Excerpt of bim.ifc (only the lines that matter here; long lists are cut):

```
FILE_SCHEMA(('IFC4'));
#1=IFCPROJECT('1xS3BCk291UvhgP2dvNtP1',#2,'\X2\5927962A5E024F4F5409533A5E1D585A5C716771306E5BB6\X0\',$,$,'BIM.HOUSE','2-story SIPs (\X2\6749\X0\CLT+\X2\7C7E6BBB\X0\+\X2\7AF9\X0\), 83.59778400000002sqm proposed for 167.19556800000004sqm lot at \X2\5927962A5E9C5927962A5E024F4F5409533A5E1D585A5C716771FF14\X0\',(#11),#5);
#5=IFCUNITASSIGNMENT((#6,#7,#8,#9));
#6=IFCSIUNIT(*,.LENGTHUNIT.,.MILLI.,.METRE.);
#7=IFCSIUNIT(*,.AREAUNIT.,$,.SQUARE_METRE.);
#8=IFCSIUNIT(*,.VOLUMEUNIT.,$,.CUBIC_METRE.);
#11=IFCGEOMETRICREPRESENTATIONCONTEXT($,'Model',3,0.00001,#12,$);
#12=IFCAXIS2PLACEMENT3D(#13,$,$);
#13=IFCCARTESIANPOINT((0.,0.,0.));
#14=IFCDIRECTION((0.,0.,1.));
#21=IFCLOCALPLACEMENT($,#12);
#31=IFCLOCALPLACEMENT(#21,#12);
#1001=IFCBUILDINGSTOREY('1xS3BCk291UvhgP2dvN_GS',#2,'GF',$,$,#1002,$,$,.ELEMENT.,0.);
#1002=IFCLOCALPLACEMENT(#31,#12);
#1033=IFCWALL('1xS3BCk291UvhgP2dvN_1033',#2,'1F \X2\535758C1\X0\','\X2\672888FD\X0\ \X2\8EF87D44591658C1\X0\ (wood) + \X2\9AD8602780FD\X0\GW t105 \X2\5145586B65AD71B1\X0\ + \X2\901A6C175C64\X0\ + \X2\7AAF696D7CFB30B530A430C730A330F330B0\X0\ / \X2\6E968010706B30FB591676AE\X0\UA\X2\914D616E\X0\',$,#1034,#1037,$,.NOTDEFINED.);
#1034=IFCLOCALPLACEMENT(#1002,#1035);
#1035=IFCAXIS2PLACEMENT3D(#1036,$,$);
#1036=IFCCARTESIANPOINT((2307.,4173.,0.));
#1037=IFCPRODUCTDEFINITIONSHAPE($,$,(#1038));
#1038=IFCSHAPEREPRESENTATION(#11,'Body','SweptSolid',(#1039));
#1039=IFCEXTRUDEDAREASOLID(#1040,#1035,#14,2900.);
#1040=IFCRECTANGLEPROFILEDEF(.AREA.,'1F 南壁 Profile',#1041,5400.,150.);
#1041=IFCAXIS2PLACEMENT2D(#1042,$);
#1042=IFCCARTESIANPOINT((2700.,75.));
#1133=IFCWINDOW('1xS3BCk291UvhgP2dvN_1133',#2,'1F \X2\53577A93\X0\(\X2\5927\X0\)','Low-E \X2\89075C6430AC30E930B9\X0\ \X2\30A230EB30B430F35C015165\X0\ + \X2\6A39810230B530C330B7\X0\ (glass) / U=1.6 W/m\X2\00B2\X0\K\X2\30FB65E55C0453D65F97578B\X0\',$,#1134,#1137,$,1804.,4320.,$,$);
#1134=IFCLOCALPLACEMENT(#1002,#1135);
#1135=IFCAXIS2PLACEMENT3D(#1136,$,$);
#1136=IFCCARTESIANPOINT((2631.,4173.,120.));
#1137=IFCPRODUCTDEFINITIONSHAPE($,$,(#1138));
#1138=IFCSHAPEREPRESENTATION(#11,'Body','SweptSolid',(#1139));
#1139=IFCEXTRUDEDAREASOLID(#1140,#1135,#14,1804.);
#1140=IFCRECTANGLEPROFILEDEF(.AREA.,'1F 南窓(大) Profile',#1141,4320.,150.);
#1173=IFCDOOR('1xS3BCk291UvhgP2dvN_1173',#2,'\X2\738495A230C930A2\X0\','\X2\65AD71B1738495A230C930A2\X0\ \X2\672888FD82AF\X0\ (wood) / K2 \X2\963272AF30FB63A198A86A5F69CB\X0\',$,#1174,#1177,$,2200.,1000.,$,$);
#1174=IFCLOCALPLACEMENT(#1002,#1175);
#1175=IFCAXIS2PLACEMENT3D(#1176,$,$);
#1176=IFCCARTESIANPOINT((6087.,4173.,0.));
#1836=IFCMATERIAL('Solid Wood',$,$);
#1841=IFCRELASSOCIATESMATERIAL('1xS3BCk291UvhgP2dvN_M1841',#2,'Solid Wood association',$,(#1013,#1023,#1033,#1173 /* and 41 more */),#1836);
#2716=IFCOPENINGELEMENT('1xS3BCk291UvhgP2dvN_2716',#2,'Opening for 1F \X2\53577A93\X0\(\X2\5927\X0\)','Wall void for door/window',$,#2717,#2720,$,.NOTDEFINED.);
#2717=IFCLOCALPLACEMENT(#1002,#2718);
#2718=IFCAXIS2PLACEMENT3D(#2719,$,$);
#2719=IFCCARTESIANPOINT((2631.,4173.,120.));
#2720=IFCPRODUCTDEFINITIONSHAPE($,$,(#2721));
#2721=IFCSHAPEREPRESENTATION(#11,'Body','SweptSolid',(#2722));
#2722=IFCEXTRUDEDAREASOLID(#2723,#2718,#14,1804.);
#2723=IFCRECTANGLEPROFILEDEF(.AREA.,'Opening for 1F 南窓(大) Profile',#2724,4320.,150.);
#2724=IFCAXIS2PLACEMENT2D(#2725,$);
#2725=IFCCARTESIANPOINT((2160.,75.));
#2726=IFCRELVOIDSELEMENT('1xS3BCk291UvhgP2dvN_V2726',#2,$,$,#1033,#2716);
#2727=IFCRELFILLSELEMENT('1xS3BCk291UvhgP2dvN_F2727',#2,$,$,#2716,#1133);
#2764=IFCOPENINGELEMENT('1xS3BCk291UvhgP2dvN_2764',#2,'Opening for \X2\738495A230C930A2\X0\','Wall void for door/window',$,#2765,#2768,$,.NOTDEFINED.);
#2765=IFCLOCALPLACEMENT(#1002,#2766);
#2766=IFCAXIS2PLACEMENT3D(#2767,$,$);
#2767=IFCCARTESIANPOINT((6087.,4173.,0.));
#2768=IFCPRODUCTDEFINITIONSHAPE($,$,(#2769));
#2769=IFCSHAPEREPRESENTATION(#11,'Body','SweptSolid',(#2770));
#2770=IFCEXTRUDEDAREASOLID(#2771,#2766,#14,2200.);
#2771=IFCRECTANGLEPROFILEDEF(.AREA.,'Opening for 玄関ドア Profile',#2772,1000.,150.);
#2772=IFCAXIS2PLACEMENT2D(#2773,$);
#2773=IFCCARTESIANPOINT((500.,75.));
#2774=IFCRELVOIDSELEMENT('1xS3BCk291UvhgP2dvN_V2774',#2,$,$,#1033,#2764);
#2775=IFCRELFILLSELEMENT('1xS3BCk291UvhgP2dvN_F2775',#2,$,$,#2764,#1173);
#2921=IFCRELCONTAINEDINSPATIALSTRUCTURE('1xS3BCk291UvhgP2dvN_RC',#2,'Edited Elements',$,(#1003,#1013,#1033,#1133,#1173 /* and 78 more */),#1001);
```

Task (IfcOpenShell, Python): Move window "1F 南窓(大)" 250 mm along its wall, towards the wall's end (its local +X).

```python
import ifcopenshell
import ifcopenshell.api.geometry
import ifcopenshell.util.placement
import ifcopenshell.util.unit

model = ifcopenshell.open("bim.ifc")
unit_scale = ifcopenshell.util.unit.calculate_unit_scale(model)

window = model.by_id(1133)
opening = window.FillsVoids[0].RelatingOpeningElement
wall = opening.VoidsElements[0].RelatingBuildingElement

wall_matrix = ifcopenshell.util.placement.get_local_placement(wall.ObjectPlacement)
shift = wall_matrix[:3, 0] * 0.25 / unit_scale
before = ifcopenshell.util.placement.get_local_placement(window.ObjectPlacement)[:3, 3].copy()

# The window is not placed relative to its opening, so move both.
for product in (opening, window):
    matrix = ifcopenshell.util.placement.get_local_placement(product.ObjectPlacement)
    matrix[:3, 3] += shift
    ifcopenshell.api.geometry.edit_object_placement(model, product=product, matrix=matrix, is_si=False)

after = ifcopenshell.util.placement.get_local_placement(window.ObjectPlacement)[:3, 3]
print("window moved by", (after - before).round(3) + 0.0)

model.write("bim-out.ifc")
```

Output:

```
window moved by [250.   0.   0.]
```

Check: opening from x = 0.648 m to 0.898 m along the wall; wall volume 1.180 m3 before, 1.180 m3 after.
